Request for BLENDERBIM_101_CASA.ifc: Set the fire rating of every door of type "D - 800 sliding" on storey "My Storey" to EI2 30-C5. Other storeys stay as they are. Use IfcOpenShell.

First a look at what the model holds.

```python
import ifcopenshell
import ifcopenshell.util.element

model = ifcopenshell.open("BLENDERBIM_101_CASA.ifc")
print(model.schema)
storey = next(s for s in model.by_type("IfcBuildingStorey") if s.Name == "My Storey")
doors = [e for e in ifcopenshell.util.element.get_decomposition(storey) if e.is_a("IfcDoor")]
seen = {}
for e in doors:
    element_type = ifcopenshell.util.element.get_type(e)
    key = (element_type.Name if element_type != e and element_type else None, ifcopenshell.util.element.get_pset(e, "Pset_DoorCommon", "FireRating"))
    seen[key] = seen.get(key, 0) + 1
for (name, value), count in sorted(seen.items(), key=str):
    print(count, "x", name, "|", value)
```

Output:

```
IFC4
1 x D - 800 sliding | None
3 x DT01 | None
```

```python
import ifcopenshell
import ifcopenshell.api.pset
import ifcopenshell.util.element

model = ifcopenshell.open("BLENDERBIM_101_CASA.ifc")

storey = next(s for s in model.by_type("IfcBuildingStorey") if s.Name == "My Storey")
doors = [e for e in ifcopenshell.util.element.get_decomposition(storey) if e.is_a("IfcDoor")]

count = 0
for e in doors:
    element_type = ifcopenshell.util.element.get_type(e)
    if element_type in (None, e) or element_type.Name != "D - 800 sliding":
        continue
    # add_pset returns the element's existing set when there is one.
    pset = ifcopenshell.api.pset.add_pset(model, product=e, name="Pset_DoorCommon")
    ifcopenshell.api.pset.edit_pset(model, pset=pset, properties={"FireRating": "EI2 30-C5"})
    count += 1

print(count, "doors updated")

model.write("BLENDERBIM_101_CASA_edited.ifc")
```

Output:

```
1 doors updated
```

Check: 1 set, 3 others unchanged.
